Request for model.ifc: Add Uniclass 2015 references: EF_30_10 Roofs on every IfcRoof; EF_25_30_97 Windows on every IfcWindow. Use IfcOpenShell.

First a look at what the model holds.

```python
import ifcopenshell

model = ifcopenshell.open("model.ifc")
print(model.schema)
print("classifications:", [c.Name for c in model.by_type("IfcClassification")])
for ifc_class in ("IfcDoor", "IfcRoof", "IfcStair", "IfcWall", "IfcWindow"):
    print(ifc_class, len(model.by_type(ifc_class)))
```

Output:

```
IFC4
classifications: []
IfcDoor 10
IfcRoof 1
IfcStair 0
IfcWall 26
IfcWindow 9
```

```python
import ifcopenshell
import ifcopenshell.api.classification

model = ifcopenshell.open("model.ifc")

system = ifcopenshell.api.classification.add_classification(model, classification="Uniclass 2015")

codes = {
    "IfcRoof": ("EF_30_10", "Roofs"),
    "IfcWindow": ("EF_25_30_97", "Windows"),
}
for ifc_class, (code, name) in codes.items():
    products = model.by_type(ifc_class)
    ifcopenshell.api.classification.add_reference(
        model, products=products, classification=system, identification=code, name=name
    )
    print(code, len(products))

model.write("model_updated.ifc")
```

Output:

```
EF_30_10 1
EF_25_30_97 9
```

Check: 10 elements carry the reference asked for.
